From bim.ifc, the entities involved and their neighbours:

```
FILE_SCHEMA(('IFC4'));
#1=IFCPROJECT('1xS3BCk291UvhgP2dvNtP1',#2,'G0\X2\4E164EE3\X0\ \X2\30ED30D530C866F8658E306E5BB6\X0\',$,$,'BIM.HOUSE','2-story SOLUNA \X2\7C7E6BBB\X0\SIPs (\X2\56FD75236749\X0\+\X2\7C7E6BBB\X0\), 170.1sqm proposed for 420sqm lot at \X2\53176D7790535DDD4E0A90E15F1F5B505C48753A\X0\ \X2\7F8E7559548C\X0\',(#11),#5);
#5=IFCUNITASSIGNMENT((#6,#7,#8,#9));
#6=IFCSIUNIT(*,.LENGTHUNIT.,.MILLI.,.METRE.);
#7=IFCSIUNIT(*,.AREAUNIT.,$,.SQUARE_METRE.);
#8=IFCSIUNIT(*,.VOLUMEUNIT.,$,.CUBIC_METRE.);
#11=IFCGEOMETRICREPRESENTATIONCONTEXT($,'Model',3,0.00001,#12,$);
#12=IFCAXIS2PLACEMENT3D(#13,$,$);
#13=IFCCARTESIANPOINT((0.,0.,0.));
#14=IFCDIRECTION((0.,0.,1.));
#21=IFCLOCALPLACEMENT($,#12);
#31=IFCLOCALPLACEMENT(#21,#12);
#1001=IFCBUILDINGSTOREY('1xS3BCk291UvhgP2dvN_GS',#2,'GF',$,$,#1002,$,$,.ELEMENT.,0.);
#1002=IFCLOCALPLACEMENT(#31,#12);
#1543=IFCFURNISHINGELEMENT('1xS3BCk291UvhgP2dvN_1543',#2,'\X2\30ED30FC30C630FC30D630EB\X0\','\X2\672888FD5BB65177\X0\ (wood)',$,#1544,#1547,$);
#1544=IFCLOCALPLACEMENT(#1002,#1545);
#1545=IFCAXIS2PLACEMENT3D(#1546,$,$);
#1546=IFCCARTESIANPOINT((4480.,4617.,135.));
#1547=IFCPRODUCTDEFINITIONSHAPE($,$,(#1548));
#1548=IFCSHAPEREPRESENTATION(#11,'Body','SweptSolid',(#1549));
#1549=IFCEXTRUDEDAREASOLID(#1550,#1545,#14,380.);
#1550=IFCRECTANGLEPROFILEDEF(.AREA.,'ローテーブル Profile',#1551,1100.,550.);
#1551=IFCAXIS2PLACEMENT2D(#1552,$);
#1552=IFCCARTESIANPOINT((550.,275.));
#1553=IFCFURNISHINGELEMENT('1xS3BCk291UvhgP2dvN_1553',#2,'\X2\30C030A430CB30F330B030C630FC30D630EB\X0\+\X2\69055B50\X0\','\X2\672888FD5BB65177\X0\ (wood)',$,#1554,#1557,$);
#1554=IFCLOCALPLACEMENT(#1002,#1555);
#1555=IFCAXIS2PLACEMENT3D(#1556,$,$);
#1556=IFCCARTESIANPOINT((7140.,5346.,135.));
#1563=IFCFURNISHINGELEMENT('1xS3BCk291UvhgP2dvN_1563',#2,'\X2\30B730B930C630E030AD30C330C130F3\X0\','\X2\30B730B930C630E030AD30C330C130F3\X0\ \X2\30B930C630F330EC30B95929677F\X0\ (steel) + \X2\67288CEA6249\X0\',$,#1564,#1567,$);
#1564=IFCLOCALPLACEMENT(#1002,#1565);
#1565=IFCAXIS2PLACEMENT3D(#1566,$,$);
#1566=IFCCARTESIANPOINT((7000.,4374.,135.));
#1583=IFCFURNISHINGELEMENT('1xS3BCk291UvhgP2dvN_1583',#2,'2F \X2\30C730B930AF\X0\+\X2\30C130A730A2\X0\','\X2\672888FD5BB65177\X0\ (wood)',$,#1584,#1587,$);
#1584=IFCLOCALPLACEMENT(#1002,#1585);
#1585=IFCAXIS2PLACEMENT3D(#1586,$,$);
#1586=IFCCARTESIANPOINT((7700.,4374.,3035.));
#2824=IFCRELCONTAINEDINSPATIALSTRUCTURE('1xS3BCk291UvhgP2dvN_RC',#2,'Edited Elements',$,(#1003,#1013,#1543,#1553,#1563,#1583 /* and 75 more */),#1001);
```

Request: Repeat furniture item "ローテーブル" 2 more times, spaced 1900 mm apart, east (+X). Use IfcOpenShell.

```python
import numpy as np
import ifcopenshell
import ifcopenshell.api.geometry
import ifcopenshell.api.root
import ifcopenshell.util.element
import ifcopenshell.util.placement

model = ifcopenshell.open("bim.ifc")


def reuse_history(source, copy):
    """copy_class also copies each property set's owner history, people and application; keep the originals."""
    for rel in copy.IsDefinedBy:
        if rel.is_a("IfcRelDefinesByProperties") and (history := rel.RelatingPropertyDefinition.OwnerHistory):
            rel.RelatingPropertyDefinition.OwnerHistory = source.OwnerHistory
            ifcopenshell.util.element.remove_deep2(model, history)


source = model.by_guid("1xS3BCk291UvhgP2dvN_1543")
base = ifcopenshell.util.placement.get_local_placement(source.ObjectPlacement)
step = np.array([1.0, 0.0, 0.0]) * 1900.0

for i in range(1, 3):
    copy = ifcopenshell.api.root.copy_class(model, product=source)
    copy.Representation = ifcopenshell.util.element.copy_deep(
        model, source.Representation, exclude=["IfcGeometricRepresentationContext", "IfcRepresentationMap"]
    )
    reuse_history(source, copy)
    matrix = base.copy()
    matrix[:3, 3] += i * step
    print("added at", matrix[:3, 3].round(3) + 0.0)
    ifcopenshell.api.geometry.edit_object_placement(model, product=copy, matrix=matrix, is_si=False)

model.write("bim_rev.ifc")
```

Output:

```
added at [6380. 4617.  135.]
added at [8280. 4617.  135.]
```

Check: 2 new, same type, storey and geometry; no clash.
